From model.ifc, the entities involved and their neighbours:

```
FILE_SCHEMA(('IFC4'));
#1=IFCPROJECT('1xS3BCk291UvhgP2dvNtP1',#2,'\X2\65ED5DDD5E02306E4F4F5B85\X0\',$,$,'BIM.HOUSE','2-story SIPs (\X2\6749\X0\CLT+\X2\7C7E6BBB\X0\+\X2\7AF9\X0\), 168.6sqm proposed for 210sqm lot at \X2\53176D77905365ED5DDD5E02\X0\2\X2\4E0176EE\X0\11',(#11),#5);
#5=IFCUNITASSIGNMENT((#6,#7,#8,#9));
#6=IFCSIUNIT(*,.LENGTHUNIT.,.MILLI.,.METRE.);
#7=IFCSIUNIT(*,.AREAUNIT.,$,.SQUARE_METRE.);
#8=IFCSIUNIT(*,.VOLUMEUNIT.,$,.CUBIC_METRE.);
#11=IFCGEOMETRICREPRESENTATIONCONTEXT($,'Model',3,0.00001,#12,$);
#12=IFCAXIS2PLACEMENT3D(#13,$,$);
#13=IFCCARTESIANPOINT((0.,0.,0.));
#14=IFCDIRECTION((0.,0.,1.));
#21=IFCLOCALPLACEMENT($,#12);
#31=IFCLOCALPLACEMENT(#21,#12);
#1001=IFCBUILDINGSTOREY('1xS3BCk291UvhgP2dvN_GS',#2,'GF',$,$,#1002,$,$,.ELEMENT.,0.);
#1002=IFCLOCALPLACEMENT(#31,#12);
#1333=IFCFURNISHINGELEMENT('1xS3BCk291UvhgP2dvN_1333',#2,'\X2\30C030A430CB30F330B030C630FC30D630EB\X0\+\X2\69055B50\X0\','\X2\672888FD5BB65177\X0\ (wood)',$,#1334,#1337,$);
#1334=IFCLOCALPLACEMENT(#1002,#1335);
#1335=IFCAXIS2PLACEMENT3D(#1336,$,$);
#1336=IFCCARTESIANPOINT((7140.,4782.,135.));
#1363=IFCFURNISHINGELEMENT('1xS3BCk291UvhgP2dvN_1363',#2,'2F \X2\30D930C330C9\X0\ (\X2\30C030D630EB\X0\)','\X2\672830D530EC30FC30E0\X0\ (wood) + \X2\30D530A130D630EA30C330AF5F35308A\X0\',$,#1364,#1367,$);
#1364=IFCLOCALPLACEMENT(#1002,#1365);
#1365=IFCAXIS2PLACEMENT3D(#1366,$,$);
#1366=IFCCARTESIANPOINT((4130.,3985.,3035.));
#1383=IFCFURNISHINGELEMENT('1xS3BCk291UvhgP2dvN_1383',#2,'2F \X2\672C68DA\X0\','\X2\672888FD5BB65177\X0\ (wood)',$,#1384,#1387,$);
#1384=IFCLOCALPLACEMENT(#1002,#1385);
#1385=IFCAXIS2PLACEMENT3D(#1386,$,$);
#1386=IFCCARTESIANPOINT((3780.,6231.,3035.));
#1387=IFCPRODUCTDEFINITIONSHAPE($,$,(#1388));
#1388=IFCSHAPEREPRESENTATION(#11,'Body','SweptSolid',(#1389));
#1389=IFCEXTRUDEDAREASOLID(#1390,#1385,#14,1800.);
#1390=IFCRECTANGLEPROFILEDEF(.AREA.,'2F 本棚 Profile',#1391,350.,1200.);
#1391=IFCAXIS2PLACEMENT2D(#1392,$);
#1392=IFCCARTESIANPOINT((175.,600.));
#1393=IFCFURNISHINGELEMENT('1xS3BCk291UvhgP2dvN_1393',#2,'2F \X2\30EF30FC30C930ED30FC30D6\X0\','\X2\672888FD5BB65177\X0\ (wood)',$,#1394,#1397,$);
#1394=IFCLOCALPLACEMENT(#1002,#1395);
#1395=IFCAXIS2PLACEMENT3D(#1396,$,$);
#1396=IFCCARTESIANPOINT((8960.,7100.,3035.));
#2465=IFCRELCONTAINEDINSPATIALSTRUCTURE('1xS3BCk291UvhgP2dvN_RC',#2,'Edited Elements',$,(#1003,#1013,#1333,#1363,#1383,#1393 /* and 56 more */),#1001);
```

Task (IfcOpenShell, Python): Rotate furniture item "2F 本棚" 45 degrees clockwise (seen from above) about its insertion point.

```python
import ifcopenshell
import ifcopenshell.api.geometry
import ifcopenshell.util.placement

model = ifcopenshell.open("model.ifc")

item = model.by_guid("1xS3BCk291UvhgP2dvN_1383")
matrix = ifcopenshell.util.placement.get_local_placement(item.ObjectPlacement)
matrix = matrix @ ifcopenshell.util.placement.rotation(-45, "Z")
ifcopenshell.api.geometry.edit_object_placement(model, product=item, matrix=matrix, is_si=False)

print(ifcopenshell.util.placement.get_local_placement(item.ObjectPlacement).round(3) + 0.0)

model.write("model_edited.ifc")
```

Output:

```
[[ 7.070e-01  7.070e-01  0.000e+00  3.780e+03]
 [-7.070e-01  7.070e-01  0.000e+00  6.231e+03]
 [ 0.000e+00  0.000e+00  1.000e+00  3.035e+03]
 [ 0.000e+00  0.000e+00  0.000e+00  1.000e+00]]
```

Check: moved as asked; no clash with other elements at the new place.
